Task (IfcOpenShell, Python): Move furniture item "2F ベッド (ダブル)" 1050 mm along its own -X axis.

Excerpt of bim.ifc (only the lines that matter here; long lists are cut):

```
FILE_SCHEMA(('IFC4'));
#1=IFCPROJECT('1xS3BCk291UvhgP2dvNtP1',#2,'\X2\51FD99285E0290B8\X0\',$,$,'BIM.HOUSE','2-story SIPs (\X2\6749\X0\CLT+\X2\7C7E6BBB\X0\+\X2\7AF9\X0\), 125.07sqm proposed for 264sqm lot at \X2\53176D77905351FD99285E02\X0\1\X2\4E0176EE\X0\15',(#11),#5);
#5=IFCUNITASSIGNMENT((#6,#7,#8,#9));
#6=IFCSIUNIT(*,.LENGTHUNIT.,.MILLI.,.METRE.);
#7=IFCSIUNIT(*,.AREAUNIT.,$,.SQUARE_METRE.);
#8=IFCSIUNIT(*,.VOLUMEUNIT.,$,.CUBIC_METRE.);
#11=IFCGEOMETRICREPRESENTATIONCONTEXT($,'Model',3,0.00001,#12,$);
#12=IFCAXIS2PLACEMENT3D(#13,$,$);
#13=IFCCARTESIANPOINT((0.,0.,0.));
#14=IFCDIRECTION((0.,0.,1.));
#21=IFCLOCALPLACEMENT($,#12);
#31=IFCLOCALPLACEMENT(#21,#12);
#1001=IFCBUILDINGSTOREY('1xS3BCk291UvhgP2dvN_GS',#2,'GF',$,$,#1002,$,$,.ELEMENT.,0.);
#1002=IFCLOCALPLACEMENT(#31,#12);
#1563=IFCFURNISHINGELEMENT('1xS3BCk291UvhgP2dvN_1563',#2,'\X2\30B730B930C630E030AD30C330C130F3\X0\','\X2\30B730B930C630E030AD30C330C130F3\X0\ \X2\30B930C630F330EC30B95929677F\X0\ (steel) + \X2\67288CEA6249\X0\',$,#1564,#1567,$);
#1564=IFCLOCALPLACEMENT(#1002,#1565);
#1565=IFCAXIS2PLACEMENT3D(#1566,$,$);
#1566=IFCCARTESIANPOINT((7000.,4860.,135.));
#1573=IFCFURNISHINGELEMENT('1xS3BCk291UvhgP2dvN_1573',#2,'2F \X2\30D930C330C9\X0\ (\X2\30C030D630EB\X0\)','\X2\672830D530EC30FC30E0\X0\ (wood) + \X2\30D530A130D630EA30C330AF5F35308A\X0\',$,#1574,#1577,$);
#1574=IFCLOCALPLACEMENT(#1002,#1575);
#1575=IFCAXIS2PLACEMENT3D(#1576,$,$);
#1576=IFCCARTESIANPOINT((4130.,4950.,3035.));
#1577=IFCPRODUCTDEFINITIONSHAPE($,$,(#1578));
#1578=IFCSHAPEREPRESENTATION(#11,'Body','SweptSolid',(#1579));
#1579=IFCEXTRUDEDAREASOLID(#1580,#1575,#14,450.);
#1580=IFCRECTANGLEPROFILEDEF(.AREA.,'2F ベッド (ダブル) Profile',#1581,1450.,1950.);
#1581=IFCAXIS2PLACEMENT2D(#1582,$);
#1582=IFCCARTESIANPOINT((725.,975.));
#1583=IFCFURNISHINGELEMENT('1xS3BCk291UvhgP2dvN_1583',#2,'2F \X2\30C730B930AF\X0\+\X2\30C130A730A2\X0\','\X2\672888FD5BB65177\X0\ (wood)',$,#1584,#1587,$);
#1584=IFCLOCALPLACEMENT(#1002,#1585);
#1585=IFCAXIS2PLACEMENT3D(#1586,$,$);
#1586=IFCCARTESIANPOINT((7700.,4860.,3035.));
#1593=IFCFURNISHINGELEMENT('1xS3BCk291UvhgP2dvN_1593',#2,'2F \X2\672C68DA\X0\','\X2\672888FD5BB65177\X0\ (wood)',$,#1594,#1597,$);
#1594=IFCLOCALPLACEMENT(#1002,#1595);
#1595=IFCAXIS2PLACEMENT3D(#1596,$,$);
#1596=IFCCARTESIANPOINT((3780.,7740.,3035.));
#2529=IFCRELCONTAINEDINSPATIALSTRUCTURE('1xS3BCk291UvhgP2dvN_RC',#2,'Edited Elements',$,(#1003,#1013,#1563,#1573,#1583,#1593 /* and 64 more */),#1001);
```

```python
import ifcopenshell
import ifcopenshell.api.geometry
import ifcopenshell.util.placement

model = ifcopenshell.open("bim.ifc")

item = model.by_guid("1xS3BCk291UvhgP2dvN_1573")
matrix = ifcopenshell.util.placement.get_local_placement(item.ObjectPlacement)
matrix[:3, 3] -= matrix[:3, 0] * 1050.0
ifcopenshell.api.geometry.edit_object_placement(model, product=item, matrix=matrix, is_si=False)

print(ifcopenshell.util.placement.get_local_placement(item.ObjectPlacement).round(3) + 0.0)

model.write("bim_rev.ifc")
```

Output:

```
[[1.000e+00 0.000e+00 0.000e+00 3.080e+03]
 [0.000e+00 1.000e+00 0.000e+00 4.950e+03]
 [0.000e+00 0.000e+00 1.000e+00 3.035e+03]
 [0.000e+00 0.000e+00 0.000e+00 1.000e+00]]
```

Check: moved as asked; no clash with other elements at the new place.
